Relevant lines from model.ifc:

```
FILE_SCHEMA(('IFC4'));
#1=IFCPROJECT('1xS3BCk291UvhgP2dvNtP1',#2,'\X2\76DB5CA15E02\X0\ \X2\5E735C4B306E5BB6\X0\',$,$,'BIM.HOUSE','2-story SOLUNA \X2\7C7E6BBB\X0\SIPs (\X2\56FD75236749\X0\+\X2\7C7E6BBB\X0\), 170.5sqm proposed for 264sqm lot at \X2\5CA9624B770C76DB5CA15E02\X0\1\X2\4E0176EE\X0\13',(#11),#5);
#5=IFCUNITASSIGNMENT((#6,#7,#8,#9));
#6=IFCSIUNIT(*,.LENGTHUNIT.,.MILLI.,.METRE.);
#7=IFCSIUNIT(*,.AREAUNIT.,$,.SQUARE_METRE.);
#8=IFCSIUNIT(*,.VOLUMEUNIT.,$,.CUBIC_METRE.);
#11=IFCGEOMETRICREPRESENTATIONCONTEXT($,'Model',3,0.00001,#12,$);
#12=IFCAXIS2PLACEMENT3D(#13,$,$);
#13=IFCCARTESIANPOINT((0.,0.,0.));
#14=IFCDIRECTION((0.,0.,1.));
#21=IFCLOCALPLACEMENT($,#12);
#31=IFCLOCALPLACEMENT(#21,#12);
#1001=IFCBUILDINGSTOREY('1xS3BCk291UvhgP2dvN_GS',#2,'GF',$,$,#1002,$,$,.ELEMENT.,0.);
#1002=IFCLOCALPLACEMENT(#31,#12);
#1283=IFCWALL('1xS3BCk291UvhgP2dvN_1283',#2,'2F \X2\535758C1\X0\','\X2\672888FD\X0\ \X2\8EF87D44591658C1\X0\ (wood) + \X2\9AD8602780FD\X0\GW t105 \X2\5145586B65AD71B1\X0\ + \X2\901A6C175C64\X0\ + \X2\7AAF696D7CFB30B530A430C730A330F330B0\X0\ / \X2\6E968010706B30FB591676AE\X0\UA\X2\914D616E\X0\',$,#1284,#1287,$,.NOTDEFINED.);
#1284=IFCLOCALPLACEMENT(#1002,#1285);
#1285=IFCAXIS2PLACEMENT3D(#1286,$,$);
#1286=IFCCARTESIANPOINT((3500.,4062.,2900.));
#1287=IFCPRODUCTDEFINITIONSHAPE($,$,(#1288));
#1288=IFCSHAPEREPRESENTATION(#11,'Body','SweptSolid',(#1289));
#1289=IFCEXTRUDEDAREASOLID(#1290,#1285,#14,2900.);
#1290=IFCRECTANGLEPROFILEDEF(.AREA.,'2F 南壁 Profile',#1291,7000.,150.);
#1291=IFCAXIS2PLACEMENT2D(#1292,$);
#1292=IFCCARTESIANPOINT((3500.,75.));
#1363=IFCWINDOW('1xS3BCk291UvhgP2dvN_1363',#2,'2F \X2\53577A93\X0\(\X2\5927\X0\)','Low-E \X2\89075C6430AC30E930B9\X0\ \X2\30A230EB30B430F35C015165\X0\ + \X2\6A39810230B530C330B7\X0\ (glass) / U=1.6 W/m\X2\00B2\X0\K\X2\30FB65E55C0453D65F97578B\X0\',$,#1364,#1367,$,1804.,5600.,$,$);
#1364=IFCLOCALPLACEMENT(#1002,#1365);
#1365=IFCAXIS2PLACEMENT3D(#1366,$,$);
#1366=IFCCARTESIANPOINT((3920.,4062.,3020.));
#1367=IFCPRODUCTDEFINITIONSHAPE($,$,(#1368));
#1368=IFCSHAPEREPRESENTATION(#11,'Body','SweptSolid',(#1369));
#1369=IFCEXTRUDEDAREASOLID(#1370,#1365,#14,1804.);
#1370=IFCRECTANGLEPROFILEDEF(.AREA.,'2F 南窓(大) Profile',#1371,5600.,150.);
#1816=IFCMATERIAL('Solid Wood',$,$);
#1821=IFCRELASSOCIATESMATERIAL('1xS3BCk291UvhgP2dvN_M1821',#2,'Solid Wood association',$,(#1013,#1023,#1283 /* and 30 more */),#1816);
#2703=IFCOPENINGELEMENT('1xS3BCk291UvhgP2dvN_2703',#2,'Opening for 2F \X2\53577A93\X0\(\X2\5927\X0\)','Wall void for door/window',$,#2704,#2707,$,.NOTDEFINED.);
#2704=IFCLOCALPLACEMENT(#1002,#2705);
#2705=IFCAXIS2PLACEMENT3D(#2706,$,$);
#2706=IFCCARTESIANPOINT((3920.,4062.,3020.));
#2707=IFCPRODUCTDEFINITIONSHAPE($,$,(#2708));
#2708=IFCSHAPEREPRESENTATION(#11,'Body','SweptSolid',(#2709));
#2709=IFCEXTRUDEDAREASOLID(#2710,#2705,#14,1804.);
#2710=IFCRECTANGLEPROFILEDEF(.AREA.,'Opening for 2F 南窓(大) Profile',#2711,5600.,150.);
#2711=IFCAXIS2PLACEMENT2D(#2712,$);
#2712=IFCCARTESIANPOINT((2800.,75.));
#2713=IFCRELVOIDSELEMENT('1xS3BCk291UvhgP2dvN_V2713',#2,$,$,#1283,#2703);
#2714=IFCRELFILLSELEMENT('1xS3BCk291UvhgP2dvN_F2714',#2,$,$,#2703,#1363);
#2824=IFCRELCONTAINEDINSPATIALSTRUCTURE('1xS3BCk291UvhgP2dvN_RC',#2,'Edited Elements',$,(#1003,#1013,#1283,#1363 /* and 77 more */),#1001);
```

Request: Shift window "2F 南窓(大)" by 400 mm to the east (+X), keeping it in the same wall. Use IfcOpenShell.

```python
import ifcopenshell
import ifcopenshell.api.geometry
import ifcopenshell.util.placement

model = ifcopenshell.open("model.ifc")

window = model.by_guid("1xS3BCk291UvhgP2dvN_1363")
opening = window.FillsVoids[0].RelatingOpeningElement
wall = opening.VoidsElements[0].RelatingBuildingElement

wall_matrix = ifcopenshell.util.placement.get_local_placement(wall.ObjectPlacement)
shift = wall_matrix[:3, 0] * 400.0
before = ifcopenshell.util.placement.get_local_placement(window.ObjectPlacement)[:3, 3].copy()

# The window is not placed relative to its opening, so move both.
for product in (opening, window):
    matrix = ifcopenshell.util.placement.get_local_placement(product.ObjectPlacement)
    matrix[:3, 3] += shift
    ifcopenshell.api.geometry.edit_object_placement(model, product=product, matrix=matrix, is_si=False)

after = ifcopenshell.util.placement.get_local_placement(window.ObjectPlacement)[:3, 3]
print("window moved by", (after - before).round(3) + 0.0)

model.write("model_rev.ifc")
```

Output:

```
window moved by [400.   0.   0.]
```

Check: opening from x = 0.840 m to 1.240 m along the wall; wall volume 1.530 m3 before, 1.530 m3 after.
